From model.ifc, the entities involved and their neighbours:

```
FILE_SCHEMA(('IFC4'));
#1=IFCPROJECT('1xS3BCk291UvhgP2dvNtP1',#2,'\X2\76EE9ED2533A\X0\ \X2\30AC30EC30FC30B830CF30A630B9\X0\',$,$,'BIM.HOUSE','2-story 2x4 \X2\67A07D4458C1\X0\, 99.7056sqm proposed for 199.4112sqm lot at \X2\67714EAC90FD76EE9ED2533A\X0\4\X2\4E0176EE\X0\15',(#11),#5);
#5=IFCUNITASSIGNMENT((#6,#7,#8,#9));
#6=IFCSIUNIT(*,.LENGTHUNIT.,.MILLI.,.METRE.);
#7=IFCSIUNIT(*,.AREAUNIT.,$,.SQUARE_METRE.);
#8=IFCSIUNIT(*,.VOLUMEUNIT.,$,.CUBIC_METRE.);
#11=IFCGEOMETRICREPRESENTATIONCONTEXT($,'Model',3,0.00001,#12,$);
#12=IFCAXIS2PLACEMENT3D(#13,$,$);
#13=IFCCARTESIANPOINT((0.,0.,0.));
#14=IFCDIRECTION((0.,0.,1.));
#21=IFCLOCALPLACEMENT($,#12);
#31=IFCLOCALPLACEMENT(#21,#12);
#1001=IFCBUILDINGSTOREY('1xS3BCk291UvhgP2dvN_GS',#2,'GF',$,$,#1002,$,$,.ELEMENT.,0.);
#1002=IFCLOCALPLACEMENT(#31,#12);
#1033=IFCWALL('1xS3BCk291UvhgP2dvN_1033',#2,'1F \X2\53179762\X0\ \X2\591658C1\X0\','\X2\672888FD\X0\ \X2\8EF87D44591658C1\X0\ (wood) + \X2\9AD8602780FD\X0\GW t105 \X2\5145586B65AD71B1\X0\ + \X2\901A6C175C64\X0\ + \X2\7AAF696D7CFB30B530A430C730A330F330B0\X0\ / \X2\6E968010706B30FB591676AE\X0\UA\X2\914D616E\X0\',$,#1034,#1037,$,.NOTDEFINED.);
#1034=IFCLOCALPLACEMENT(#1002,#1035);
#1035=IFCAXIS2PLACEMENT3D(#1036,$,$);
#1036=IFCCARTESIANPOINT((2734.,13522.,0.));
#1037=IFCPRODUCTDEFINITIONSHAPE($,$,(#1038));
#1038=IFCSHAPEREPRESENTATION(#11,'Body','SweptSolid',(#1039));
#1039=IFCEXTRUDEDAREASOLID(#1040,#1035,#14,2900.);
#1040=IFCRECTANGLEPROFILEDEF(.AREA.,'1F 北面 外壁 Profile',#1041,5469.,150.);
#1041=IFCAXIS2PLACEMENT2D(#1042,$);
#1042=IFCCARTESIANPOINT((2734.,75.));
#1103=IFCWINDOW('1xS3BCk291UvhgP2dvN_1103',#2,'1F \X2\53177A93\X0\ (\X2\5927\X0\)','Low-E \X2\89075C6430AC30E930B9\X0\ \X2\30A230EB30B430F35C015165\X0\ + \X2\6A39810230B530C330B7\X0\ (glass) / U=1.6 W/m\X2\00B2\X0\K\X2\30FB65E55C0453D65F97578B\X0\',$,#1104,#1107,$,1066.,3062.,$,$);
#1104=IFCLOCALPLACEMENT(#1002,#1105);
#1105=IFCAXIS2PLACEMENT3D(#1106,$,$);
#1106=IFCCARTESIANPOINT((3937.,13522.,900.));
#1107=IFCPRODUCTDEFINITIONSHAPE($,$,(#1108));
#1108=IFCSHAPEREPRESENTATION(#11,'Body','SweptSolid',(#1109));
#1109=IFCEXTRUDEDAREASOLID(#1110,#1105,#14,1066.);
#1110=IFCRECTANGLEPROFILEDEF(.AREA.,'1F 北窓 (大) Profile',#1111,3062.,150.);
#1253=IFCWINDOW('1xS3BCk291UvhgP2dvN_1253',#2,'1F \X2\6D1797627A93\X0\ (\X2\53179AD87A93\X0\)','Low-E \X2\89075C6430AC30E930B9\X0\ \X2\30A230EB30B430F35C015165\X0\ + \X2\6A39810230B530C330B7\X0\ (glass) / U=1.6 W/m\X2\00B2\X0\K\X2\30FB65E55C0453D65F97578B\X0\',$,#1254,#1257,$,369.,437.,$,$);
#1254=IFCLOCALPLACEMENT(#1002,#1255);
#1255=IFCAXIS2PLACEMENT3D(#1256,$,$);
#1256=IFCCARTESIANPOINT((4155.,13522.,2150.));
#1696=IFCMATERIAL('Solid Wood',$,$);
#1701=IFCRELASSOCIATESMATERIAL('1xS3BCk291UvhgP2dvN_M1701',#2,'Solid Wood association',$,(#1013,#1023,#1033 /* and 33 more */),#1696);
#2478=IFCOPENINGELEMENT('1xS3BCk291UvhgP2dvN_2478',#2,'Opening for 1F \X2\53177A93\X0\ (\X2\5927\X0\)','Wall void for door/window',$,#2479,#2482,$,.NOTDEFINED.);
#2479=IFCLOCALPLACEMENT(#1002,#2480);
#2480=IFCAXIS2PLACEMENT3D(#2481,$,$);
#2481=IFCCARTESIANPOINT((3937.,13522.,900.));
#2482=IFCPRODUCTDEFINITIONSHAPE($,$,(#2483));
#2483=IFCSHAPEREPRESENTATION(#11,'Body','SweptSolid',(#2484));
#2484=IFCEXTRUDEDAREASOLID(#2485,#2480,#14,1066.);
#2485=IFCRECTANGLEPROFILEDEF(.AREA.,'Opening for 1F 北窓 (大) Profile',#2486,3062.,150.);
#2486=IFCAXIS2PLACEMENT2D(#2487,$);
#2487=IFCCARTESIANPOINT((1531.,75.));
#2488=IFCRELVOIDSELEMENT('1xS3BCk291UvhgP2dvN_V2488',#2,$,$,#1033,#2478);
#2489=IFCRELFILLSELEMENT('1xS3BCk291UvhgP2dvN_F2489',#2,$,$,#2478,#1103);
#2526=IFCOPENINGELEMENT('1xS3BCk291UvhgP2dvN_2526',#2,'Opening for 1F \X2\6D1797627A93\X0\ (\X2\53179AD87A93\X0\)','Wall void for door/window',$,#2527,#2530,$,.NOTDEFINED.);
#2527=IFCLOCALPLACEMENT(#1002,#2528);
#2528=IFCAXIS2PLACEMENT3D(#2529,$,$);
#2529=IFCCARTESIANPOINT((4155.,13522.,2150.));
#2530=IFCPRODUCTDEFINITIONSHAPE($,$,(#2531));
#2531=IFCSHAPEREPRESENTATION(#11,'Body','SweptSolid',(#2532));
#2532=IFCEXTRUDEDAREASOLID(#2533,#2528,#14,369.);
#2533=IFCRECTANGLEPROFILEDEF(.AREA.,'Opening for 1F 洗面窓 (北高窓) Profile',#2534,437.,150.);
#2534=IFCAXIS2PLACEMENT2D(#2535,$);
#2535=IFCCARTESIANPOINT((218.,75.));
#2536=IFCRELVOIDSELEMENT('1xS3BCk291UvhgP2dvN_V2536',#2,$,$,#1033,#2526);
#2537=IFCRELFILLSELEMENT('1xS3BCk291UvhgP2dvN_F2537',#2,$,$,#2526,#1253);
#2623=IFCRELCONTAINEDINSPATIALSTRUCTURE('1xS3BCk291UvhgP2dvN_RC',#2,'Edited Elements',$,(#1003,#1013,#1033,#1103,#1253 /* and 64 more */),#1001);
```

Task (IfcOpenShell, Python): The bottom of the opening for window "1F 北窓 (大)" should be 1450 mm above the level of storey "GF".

```python
import numpy as np
import ifcopenshell
import ifcopenshell.api.geometry
import ifcopenshell.geom
import ifcopenshell.util.element
import ifcopenshell.util.placement
import ifcopenshell.util.shape
import ifcopenshell.util.unit

model = ifcopenshell.open("model.ifc")
unit_scale = ifcopenshell.util.unit.calculate_unit_scale(model)

window = model.by_id(1103)
opening = window.FillsVoids[0].RelatingOpeningElement
storey = ifcopenshell.util.element.get_container(window, ifc_class="IfcBuildingStorey")
level = ifcopenshell.util.placement.get_local_placement(storey.ObjectPlacement)[2, 3]

# The opening's origin need not be at the sill, so measure its lowest point.
shape = ifcopenshell.geom.create_shape(ifcopenshell.geom.settings(), opening)
bottom = ifcopenshell.util.shape.get_shape_bottom_elevation(shape, shape.geometry) / unit_scale
dz = level + 1450.0 - bottom

shift = np.array([0.0, 0.0, dz])
# The window is not placed relative to its opening, so move both.
for product in (opening, window):
    matrix = ifcopenshell.util.placement.get_local_placement(product.ObjectPlacement)
    matrix[:3, 3] += shift
    ifcopenshell.api.geometry.edit_object_placement(model, product=product, matrix=matrix, is_si=False)

print(f"moved by {dz * unit_scale:+.3f} m")

model.write("model_updated.ifc")
```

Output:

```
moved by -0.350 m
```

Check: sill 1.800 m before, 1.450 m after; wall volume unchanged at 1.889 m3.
